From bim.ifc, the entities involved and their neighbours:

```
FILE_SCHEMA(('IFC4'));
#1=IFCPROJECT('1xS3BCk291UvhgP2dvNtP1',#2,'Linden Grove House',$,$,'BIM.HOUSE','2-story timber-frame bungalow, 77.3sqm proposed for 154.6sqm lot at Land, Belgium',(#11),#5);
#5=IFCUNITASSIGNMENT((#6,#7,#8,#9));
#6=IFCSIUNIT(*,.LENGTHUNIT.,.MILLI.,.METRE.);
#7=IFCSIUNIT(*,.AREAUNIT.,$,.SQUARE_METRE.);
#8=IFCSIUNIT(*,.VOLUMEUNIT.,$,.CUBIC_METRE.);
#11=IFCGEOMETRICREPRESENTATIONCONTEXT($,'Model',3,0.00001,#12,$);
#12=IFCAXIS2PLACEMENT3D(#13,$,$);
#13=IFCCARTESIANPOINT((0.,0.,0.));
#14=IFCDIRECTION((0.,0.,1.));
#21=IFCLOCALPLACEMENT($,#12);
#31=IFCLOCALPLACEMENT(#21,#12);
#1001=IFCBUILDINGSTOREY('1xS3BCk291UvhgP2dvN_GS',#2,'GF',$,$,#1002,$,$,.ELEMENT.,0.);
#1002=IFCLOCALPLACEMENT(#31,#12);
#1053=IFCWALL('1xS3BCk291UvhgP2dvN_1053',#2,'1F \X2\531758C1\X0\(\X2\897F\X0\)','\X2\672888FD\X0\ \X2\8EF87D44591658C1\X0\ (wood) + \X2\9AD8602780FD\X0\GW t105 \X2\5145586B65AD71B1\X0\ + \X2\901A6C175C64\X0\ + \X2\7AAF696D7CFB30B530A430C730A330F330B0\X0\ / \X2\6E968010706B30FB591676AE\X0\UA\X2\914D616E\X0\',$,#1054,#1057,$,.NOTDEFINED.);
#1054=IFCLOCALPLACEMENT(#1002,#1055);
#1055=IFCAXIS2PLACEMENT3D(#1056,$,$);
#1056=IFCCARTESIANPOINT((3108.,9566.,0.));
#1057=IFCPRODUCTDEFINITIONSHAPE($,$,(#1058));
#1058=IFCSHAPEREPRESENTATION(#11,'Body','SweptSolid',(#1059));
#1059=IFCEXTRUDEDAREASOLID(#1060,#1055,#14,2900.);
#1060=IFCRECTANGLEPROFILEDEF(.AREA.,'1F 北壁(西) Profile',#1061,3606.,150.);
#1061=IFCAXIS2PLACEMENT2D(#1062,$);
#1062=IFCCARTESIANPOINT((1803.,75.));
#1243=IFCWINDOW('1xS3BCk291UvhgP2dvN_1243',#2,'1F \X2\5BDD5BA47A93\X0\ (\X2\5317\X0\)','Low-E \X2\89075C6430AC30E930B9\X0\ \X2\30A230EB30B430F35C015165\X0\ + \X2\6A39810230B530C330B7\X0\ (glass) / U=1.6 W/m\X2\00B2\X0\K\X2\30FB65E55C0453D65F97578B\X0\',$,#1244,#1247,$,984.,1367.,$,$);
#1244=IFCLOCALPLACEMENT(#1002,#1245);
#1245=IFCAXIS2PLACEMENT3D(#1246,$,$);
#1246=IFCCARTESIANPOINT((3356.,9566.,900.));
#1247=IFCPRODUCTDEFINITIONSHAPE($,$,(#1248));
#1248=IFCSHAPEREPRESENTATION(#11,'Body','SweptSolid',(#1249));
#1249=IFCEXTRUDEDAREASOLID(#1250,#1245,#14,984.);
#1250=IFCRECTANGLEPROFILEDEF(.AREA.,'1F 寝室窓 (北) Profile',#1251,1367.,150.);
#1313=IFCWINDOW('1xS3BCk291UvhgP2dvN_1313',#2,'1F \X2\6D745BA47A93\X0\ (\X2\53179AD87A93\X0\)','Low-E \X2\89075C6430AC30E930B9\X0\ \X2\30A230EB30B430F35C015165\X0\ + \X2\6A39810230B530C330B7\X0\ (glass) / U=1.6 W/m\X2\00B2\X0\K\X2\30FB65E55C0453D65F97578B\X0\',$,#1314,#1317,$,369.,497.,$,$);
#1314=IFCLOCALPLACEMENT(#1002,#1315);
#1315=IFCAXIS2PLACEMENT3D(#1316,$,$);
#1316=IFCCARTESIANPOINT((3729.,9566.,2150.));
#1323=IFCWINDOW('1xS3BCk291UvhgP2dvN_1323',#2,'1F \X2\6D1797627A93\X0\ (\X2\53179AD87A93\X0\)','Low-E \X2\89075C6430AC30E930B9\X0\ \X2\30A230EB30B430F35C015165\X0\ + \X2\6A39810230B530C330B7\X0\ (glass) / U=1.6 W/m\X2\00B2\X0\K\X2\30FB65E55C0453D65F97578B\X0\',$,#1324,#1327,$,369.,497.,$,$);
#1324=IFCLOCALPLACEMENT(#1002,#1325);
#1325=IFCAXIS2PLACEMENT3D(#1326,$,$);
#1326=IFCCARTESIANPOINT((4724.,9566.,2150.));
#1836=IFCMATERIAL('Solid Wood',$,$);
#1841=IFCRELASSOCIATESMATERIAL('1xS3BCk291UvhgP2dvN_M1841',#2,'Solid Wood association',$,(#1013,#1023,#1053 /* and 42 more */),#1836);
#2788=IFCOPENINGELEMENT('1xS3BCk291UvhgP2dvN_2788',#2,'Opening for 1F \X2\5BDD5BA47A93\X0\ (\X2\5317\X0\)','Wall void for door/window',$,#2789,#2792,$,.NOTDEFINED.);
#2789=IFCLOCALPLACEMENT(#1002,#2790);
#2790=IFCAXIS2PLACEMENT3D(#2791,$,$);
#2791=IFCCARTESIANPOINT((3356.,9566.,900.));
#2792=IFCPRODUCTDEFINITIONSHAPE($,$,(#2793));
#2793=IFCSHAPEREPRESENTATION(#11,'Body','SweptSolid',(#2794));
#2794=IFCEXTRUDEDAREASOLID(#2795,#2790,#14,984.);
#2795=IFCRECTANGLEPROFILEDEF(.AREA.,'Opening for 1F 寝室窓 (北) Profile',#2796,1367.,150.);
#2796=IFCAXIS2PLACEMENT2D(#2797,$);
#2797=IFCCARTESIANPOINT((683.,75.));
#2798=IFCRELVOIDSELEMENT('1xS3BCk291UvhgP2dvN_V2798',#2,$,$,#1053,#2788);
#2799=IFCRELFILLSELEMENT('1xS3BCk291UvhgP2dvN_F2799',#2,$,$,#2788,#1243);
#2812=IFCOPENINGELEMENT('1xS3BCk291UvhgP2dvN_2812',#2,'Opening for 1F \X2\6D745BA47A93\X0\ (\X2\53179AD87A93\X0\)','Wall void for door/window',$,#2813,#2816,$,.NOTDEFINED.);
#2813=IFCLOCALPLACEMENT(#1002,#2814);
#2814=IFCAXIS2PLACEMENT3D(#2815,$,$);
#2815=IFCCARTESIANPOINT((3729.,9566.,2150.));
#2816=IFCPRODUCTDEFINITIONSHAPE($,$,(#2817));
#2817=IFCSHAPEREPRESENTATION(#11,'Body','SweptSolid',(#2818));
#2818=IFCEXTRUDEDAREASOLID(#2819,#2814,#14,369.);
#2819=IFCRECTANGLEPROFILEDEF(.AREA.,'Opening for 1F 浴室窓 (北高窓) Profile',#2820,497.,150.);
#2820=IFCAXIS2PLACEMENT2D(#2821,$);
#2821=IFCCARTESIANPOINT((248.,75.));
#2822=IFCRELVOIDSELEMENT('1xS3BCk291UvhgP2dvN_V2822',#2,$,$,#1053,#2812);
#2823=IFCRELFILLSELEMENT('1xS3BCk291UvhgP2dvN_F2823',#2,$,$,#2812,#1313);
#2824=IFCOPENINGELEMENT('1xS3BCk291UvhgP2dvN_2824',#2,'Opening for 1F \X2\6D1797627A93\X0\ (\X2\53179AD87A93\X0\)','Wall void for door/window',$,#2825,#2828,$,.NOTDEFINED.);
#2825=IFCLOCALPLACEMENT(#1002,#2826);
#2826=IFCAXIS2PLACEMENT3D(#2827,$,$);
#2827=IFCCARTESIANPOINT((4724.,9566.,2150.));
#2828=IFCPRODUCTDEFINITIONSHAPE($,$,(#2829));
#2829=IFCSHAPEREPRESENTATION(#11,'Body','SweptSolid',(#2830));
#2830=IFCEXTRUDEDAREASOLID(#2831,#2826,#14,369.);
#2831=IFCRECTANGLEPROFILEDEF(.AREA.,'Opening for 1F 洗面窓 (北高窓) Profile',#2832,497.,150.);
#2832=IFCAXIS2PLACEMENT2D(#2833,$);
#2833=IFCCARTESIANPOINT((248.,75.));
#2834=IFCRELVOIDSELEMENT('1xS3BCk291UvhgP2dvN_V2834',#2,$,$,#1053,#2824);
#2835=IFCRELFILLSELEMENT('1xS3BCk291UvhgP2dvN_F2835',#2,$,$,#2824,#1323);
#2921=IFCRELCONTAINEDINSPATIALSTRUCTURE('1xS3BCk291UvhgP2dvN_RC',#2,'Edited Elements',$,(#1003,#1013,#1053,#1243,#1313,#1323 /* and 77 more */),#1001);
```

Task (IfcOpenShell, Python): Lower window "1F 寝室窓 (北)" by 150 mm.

```python
import numpy as np
import ifcopenshell
import ifcopenshell.api.geometry
import ifcopenshell.util.placement
import ifcopenshell.util.unit

model = ifcopenshell.open("bim.ifc")
unit_scale = ifcopenshell.util.unit.calculate_unit_scale(model)

window = model.by_guid("1xS3BCk291UvhgP2dvN_1243")
opening = window.FillsVoids[0].RelatingOpeningElement
dz = -0.15 / unit_scale

shift = np.array([0.0, 0.0, dz])
# The window is not placed relative to its opening, so move both.
for product in (opening, window):
    matrix = ifcopenshell.util.placement.get_local_placement(product.ObjectPlacement)
    matrix[:3, 3] += shift
    ifcopenshell.api.geometry.edit_object_placement(model, product=product, matrix=matrix, is_si=False)

print(f"moved by {dz * unit_scale:+.3f} m")

model.write("bim_edited.ifc")
```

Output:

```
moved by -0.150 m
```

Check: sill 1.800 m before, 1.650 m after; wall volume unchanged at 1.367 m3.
